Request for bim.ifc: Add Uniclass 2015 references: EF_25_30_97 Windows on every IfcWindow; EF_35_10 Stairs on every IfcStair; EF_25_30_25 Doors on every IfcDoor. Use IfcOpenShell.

First a look at what the model holds.

```python
import ifcopenshell

model = ifcopenshell.open("bim.ifc")
print(model.schema)
print("classifications:", [c.Name for c in model.by_type("IfcClassification")])
for ifc_class in ("IfcDoor", "IfcRoof", "IfcStair", "IfcWall", "IfcWindow"):
    print(ifc_class, len(model.by_type(ifc_class)))
```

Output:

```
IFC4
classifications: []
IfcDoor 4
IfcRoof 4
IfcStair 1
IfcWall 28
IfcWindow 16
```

```python
import ifcopenshell
import ifcopenshell.api.classification

model = ifcopenshell.open("bim.ifc")

system = ifcopenshell.api.classification.add_classification(model, classification="Uniclass 2015")

codes = {
    "IfcWindow": ("EF_25_30_97", "Windows"),
    "IfcStair": ("EF_35_10", "Stairs"),
    "IfcDoor": ("EF_25_30_25", "Doors"),
}
for ifc_class, (code, name) in codes.items():
    products = model.by_type(ifc_class)
    ifcopenshell.api.classification.add_reference(
        model, products=products, classification=system, identification=code, name=name
    )
    print(code, len(products))

model.write("bim_rev.ifc")
```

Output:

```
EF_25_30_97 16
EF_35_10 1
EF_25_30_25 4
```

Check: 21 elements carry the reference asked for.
